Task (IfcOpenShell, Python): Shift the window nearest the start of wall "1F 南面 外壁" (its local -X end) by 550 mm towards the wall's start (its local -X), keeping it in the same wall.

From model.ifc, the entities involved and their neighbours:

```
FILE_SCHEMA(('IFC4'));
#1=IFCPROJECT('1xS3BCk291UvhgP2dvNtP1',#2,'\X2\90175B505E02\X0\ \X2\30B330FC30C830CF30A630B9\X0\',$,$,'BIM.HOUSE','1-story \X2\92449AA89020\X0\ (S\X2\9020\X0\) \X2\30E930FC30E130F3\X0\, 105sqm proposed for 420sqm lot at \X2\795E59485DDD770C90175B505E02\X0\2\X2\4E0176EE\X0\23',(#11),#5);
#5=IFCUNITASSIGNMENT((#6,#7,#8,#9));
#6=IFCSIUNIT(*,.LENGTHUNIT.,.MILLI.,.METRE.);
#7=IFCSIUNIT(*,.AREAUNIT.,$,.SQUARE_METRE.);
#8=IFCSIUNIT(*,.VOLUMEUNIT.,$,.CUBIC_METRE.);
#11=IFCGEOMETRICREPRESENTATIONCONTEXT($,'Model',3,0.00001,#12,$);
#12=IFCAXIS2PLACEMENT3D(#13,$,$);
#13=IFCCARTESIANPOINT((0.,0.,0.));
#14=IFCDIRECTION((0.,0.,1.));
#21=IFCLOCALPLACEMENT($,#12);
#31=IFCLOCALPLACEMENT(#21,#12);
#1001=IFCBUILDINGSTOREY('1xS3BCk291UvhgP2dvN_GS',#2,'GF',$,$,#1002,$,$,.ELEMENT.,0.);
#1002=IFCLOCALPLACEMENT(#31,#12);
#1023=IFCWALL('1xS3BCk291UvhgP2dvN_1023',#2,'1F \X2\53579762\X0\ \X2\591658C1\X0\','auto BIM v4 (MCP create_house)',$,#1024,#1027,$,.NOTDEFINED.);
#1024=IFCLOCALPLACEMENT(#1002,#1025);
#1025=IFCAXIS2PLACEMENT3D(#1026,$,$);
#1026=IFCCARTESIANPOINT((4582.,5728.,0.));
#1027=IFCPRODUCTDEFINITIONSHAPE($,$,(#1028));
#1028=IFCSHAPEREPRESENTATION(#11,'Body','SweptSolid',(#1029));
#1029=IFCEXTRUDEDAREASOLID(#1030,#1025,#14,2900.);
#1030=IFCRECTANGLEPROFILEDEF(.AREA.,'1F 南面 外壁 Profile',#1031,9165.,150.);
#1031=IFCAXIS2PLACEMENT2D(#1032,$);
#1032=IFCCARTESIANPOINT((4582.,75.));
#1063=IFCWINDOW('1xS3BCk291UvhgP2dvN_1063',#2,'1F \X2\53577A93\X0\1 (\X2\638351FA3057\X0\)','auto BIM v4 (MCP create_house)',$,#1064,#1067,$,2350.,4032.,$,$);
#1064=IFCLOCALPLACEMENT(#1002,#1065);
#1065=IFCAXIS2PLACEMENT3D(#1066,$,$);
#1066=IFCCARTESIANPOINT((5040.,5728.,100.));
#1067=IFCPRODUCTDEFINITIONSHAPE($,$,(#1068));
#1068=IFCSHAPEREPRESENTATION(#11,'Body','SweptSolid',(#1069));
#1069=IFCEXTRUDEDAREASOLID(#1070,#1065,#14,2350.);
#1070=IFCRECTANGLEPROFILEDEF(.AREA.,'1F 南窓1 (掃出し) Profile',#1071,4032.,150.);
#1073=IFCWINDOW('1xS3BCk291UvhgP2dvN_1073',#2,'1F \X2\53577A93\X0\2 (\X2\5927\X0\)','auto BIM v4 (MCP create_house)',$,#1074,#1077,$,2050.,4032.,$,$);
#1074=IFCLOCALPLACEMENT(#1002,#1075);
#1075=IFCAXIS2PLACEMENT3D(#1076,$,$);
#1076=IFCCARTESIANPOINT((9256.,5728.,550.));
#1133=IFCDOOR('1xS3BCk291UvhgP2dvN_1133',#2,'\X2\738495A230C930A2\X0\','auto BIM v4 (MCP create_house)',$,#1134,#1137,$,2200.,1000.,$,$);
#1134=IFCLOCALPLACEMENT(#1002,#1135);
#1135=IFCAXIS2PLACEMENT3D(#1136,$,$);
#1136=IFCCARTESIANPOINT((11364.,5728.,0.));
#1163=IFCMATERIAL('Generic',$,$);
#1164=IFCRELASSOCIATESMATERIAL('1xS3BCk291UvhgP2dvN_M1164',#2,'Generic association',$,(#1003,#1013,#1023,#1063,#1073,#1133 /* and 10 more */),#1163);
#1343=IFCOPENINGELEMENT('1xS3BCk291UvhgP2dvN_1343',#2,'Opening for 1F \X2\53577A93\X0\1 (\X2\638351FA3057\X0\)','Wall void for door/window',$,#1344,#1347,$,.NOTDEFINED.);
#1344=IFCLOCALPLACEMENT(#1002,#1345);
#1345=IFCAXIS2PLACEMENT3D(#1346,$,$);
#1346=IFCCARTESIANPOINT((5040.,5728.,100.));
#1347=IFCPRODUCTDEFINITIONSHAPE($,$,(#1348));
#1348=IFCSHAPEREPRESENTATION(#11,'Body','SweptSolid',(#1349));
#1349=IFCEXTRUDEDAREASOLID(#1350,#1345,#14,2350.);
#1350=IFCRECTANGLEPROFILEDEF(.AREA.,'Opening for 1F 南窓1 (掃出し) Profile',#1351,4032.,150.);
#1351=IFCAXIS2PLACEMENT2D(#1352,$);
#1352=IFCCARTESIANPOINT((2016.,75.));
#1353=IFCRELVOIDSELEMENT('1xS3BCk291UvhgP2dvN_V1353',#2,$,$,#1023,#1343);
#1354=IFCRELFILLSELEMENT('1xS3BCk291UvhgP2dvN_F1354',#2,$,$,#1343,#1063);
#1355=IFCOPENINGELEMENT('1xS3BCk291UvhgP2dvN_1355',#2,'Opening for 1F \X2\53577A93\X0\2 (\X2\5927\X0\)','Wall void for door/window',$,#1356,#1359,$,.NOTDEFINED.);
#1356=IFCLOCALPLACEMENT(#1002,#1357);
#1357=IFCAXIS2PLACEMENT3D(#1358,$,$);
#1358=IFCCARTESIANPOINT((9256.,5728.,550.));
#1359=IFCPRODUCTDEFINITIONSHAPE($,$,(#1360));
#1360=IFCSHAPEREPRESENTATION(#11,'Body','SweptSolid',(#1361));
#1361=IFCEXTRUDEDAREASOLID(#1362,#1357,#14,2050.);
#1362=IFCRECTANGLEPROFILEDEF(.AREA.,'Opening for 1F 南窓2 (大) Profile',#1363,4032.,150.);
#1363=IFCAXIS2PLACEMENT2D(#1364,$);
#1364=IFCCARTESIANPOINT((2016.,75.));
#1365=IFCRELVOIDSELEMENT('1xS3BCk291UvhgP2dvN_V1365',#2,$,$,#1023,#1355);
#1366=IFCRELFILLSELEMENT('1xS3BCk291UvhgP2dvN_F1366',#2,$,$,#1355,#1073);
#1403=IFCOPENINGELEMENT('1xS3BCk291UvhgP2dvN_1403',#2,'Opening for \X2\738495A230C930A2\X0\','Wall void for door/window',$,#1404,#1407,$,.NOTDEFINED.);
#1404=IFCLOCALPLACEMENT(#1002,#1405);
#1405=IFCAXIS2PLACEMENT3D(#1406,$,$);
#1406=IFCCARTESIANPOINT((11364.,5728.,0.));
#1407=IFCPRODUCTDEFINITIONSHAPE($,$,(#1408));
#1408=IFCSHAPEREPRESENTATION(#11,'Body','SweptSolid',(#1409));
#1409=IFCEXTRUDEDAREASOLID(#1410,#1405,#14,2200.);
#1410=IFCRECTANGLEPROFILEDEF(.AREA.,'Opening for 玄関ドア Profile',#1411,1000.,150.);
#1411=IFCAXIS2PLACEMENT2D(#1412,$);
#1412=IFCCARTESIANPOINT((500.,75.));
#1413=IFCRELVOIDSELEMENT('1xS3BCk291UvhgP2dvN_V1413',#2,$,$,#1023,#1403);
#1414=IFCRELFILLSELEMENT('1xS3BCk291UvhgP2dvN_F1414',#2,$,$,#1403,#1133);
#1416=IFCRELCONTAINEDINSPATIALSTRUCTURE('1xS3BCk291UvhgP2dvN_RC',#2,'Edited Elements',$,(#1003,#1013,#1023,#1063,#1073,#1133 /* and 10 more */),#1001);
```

```python
import ifcopenshell
import ifcopenshell.api.geometry
import ifcopenshell.util.placement
import ifcopenshell.util.unit

model = ifcopenshell.open("model.ifc")
unit_scale = ifcopenshell.util.unit.calculate_unit_scale(model)

window = model.by_guid("1xS3BCk291UvhgP2dvN_1063")
opening = window.FillsVoids[0].RelatingOpeningElement
wall = opening.VoidsElements[0].RelatingBuildingElement

wall_matrix = ifcopenshell.util.placement.get_local_placement(wall.ObjectPlacement)
shift = wall_matrix[:3, 0] * -0.55 / unit_scale
before = ifcopenshell.util.placement.get_local_placement(window.ObjectPlacement)[:3, 3].copy()

# The window is not placed relative to its opening, so move both.
for product in (opening, window):
    matrix = ifcopenshell.util.placement.get_local_placement(product.ObjectPlacement)
    matrix[:3, 3] += shift
    ifcopenshell.api.geometry.edit_object_placement(model, product=product, matrix=matrix, is_si=False)

after = ifcopenshell.util.placement.get_local_placement(window.ObjectPlacement)[:3, 3]
print("window moved by", (after - before).round(3) + 0.0)

model.write("model_edited.ifc")
```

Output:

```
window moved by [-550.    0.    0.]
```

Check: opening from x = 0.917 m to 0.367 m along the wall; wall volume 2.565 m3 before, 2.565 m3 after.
